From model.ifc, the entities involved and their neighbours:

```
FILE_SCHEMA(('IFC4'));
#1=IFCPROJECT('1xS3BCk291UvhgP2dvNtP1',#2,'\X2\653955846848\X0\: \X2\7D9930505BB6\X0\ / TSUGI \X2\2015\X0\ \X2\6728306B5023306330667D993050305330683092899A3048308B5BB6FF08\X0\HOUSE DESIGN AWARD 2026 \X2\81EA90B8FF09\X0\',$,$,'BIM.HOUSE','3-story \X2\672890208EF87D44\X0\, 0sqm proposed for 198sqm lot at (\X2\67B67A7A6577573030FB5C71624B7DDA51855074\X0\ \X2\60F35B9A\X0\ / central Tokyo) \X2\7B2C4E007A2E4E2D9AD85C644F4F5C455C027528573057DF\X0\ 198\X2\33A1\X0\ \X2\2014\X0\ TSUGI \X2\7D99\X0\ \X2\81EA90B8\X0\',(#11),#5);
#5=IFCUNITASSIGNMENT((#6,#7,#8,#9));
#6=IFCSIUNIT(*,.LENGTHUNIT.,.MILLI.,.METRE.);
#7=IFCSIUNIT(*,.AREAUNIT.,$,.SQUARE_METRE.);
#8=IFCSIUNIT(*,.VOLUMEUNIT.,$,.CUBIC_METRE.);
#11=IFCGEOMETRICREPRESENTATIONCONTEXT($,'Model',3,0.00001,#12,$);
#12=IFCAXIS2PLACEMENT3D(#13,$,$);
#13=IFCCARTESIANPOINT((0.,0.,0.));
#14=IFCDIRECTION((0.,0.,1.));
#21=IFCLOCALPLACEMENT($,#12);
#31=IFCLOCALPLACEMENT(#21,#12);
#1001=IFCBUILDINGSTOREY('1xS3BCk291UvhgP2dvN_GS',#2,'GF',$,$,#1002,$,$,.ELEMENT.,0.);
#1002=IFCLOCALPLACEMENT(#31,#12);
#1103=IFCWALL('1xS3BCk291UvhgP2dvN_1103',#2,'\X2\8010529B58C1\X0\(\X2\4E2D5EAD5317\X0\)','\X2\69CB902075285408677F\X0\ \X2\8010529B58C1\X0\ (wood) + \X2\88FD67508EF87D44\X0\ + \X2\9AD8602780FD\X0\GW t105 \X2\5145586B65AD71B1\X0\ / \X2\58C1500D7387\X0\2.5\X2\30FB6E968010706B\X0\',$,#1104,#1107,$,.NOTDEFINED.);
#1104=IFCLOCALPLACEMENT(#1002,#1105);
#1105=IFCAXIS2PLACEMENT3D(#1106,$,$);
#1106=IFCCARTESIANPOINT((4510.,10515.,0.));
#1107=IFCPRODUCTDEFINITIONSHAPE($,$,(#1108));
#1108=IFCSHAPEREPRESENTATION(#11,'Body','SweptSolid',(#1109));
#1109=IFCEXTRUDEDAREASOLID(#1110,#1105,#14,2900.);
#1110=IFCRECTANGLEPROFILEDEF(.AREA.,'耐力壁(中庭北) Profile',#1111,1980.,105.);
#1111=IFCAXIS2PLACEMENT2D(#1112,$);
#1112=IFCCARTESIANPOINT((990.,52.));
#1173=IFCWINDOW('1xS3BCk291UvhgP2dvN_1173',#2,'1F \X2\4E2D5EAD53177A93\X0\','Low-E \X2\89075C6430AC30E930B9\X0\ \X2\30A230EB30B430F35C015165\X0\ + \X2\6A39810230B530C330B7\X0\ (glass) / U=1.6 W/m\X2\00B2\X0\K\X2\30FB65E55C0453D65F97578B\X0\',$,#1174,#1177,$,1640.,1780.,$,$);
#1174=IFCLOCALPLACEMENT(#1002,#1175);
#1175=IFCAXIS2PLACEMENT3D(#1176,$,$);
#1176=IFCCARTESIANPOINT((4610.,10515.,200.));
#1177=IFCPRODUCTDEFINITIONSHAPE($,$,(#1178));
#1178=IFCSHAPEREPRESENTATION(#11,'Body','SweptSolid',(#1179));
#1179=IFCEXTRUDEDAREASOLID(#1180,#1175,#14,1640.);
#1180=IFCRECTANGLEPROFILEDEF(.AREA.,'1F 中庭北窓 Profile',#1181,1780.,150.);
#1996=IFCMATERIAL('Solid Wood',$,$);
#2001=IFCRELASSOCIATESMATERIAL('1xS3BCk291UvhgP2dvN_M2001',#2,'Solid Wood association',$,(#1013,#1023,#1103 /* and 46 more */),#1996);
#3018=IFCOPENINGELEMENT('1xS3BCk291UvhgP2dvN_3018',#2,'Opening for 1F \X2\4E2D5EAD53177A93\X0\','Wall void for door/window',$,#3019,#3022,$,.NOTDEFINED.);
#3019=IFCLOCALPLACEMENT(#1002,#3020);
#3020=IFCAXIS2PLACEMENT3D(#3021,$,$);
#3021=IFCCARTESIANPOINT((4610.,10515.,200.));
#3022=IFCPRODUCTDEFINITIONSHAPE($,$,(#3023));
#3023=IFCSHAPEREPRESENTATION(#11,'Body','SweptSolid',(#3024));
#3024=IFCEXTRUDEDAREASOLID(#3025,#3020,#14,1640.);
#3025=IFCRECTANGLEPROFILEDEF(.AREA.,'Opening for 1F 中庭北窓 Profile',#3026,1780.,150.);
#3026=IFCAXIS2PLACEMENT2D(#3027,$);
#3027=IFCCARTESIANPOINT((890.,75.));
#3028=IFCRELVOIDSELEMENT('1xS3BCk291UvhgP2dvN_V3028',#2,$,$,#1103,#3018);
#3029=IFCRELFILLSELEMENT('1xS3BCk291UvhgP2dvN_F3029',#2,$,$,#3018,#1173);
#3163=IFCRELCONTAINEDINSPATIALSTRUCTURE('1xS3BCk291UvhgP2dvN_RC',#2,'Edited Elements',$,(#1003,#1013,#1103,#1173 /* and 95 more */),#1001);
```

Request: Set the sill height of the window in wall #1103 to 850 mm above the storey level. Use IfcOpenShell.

```python
import numpy as np
import ifcopenshell
import ifcopenshell.api.geometry
import ifcopenshell.geom
import ifcopenshell.util.element
import ifcopenshell.util.placement
import ifcopenshell.util.shape
import ifcopenshell.util.unit

model = ifcopenshell.open("model.ifc")
unit_scale = ifcopenshell.util.unit.calculate_unit_scale(model)

window = model.by_id(1173)
opening = window.FillsVoids[0].RelatingOpeningElement
storey = ifcopenshell.util.element.get_container(window, ifc_class="IfcBuildingStorey")
level = ifcopenshell.util.placement.get_local_placement(storey.ObjectPlacement)[2, 3]

# The opening's origin need not be at the sill, so measure its lowest point.
shape = ifcopenshell.geom.create_shape(ifcopenshell.geom.settings(), opening)
bottom = ifcopenshell.util.shape.get_shape_bottom_elevation(shape, shape.geometry) / unit_scale
dz = level + 850.0 - bottom

shift = np.array([0.0, 0.0, dz])
# The window is not placed relative to its opening, so move both.
for product in (opening, window):
    matrix = ifcopenshell.util.placement.get_local_placement(product.ObjectPlacement)
    matrix[:3, 3] += shift
    ifcopenshell.api.geometry.edit_object_placement(model, product=product, matrix=matrix, is_si=False)

print(f"moved by {dz * unit_scale:+.3f} m")

model.write("model_updated.ifc")
```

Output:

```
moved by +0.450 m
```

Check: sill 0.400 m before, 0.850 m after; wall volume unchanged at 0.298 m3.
